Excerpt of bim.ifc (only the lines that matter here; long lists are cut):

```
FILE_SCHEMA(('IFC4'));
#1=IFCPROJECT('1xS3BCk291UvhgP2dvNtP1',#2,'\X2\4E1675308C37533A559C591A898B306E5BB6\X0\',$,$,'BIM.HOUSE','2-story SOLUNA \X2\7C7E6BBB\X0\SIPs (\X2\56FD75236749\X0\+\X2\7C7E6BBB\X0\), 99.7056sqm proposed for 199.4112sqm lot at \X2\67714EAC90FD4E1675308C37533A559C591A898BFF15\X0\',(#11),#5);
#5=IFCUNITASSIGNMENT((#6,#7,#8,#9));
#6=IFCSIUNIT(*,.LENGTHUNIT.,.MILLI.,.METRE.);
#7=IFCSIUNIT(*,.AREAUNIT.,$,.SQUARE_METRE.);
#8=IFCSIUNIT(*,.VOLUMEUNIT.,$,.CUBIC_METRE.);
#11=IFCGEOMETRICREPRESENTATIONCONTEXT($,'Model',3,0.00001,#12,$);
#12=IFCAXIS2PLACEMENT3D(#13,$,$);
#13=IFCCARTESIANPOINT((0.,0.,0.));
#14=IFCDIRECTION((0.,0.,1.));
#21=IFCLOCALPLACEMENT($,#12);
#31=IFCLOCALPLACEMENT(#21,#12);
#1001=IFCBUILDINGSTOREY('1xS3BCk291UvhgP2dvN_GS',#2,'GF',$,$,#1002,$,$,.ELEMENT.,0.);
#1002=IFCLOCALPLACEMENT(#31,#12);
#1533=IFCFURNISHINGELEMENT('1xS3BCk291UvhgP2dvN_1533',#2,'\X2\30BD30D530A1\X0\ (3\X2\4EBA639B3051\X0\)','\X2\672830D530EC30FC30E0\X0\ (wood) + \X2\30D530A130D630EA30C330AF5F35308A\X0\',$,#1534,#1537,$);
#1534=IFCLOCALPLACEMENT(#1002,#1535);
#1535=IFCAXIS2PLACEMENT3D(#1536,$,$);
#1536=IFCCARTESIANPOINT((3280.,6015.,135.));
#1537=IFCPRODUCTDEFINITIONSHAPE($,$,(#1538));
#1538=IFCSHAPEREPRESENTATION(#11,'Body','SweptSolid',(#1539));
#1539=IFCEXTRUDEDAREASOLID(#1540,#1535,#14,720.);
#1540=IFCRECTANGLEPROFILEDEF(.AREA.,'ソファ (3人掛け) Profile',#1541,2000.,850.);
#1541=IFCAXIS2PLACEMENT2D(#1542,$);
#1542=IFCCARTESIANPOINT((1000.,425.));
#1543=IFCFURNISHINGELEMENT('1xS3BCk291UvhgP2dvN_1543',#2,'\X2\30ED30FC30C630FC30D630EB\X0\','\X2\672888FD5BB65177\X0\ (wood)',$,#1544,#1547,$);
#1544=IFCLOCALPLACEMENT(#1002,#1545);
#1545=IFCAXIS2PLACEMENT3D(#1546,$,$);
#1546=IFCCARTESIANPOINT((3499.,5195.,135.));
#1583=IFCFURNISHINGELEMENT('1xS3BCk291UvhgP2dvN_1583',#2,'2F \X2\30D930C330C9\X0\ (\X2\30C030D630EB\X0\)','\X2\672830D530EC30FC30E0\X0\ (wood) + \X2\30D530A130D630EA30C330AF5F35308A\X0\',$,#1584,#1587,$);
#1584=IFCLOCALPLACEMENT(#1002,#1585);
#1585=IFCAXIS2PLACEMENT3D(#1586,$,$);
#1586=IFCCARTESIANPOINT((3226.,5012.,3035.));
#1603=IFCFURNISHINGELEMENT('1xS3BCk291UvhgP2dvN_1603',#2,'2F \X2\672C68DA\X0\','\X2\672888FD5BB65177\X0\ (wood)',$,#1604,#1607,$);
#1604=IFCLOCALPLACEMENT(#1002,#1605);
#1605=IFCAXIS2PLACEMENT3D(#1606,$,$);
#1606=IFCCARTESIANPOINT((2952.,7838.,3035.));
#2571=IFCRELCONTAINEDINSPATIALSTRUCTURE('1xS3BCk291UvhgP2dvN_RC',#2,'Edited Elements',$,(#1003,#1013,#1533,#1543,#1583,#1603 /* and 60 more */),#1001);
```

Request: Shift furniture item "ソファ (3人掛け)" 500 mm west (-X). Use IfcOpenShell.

```python
import ifcopenshell
import ifcopenshell.api.geometry
import ifcopenshell.util.placement
import ifcopenshell.util.unit

model = ifcopenshell.open("bim.ifc")
unit_scale = ifcopenshell.util.unit.calculate_unit_scale(model)

item = model.by_guid("1xS3BCk291UvhgP2dvN_1533")
matrix = ifcopenshell.util.placement.get_local_placement(item.ObjectPlacement)
matrix[0, 3] -= 0.5 / unit_scale
ifcopenshell.api.geometry.edit_object_placement(model, product=item, matrix=matrix, is_si=False)

print(ifcopenshell.util.placement.get_local_placement(item.ObjectPlacement).round(3) + 0.0)

model.write("bim_v2.ifc")
```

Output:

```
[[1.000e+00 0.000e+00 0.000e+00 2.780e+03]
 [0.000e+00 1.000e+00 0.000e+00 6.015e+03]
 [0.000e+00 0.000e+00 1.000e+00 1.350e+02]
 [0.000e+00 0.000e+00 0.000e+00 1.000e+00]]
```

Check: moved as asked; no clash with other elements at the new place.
